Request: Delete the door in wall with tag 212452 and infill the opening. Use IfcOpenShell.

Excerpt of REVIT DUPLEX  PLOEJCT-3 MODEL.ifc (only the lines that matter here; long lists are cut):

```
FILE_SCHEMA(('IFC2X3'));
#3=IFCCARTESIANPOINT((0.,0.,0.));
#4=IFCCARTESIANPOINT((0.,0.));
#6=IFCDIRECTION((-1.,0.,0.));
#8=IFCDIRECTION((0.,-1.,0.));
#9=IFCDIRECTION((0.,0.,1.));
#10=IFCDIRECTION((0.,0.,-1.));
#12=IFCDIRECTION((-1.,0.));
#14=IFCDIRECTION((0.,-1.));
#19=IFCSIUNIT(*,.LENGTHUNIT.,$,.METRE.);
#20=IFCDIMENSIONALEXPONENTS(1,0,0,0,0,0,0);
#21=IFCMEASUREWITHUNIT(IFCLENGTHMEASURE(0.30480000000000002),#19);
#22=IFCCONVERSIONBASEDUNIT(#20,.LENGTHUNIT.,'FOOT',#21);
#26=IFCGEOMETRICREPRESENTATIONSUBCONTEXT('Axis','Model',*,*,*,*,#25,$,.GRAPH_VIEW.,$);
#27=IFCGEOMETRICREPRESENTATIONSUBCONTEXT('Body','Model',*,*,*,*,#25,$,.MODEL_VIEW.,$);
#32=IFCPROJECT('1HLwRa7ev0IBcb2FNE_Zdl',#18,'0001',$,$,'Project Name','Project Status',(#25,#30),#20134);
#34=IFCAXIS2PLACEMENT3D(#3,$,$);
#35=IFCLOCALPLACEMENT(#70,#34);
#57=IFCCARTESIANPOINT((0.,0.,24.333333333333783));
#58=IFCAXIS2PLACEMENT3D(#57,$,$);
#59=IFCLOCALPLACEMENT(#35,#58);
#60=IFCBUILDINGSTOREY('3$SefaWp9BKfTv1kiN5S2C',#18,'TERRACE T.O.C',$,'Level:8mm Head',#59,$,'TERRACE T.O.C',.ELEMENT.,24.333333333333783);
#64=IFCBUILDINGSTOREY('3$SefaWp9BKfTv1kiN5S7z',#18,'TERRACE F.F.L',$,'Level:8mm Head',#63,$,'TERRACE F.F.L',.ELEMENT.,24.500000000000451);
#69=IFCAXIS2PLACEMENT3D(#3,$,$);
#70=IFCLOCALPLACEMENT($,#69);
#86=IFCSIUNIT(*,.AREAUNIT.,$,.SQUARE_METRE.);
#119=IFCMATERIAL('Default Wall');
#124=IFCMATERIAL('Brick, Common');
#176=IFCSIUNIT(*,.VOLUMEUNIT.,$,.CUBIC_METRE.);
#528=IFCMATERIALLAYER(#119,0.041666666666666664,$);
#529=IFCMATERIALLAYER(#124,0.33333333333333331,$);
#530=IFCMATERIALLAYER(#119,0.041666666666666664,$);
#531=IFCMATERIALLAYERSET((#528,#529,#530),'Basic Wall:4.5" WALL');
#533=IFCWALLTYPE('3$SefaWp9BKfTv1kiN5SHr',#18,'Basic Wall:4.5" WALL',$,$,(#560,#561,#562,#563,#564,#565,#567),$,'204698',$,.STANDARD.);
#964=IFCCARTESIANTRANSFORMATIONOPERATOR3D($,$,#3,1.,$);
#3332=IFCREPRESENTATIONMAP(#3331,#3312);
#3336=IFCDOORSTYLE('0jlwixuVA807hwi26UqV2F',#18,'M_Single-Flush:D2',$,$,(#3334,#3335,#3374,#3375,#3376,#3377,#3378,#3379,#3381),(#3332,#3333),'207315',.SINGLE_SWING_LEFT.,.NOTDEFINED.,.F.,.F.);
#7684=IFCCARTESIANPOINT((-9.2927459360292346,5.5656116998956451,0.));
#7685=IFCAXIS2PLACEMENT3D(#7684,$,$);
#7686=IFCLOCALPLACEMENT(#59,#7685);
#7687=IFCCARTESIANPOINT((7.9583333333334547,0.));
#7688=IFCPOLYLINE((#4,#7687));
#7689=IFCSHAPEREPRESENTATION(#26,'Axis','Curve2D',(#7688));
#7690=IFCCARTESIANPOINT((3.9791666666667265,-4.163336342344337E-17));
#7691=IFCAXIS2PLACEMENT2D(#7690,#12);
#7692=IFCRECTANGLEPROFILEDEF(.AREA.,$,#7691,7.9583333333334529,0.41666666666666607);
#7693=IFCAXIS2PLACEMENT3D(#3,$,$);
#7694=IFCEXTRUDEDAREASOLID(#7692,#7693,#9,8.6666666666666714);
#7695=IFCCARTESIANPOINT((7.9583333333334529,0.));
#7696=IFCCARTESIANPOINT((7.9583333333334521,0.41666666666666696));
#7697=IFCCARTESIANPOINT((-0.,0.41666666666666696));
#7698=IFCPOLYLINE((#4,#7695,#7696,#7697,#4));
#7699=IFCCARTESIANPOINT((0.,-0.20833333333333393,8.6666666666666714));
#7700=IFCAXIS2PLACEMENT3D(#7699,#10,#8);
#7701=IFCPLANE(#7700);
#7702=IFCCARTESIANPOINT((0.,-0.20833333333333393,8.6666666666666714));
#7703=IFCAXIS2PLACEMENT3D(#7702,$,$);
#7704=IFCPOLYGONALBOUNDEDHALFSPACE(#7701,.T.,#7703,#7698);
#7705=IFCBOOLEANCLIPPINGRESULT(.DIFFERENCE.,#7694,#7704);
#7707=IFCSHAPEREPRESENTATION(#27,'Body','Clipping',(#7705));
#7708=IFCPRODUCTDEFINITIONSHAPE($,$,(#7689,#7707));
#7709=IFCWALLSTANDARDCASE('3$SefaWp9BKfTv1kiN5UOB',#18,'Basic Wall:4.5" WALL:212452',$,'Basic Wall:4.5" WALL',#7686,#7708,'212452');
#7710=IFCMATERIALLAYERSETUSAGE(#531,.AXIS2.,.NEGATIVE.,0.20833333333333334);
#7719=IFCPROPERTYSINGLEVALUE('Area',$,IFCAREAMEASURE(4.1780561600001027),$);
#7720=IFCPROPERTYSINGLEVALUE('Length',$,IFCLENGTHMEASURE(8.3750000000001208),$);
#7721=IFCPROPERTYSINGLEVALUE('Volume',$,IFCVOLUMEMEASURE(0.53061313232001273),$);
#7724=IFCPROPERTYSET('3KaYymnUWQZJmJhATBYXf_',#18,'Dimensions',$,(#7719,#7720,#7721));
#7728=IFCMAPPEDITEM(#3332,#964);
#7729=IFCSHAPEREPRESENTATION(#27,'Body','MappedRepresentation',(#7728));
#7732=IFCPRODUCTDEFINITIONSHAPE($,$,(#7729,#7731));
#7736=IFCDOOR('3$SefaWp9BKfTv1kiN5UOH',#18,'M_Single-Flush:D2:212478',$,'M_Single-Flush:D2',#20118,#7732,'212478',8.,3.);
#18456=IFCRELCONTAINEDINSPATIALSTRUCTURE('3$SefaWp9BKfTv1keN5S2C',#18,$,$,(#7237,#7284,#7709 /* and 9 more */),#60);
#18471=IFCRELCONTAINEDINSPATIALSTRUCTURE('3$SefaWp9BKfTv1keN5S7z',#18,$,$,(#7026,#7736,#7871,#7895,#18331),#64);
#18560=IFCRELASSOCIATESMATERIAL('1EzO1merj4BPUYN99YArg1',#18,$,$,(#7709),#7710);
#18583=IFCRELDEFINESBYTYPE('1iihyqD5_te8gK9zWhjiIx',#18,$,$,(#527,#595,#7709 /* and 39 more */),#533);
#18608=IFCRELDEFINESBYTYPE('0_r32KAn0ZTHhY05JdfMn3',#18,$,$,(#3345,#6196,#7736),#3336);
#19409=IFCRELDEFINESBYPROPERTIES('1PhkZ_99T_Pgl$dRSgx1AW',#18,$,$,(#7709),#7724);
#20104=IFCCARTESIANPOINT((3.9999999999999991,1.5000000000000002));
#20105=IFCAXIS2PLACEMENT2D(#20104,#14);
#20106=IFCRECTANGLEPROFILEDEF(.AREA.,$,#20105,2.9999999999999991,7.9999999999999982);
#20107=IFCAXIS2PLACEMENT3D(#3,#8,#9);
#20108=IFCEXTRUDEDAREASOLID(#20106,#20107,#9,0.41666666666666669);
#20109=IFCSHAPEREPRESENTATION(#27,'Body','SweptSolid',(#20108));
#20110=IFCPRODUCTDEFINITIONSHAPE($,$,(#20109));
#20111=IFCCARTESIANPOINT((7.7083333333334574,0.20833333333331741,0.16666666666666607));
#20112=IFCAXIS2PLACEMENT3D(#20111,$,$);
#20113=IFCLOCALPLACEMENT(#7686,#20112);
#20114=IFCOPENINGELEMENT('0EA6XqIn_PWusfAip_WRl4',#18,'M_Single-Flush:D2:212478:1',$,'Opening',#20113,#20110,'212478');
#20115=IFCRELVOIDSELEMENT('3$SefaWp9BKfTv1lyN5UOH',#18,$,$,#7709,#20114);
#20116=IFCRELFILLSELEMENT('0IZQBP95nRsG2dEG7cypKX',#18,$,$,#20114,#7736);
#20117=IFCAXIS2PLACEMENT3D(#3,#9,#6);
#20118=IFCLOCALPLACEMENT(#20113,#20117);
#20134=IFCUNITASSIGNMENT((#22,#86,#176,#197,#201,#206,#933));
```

```python
import ifcopenshell
import ifcopenshell.api.feature
import ifcopenshell.api.pset
import ifcopenshell.api.root
import ifcopenshell.geom
import ifcopenshell.util.element
import ifcopenshell.util.shape
import ifcopenshell.util.unit

model = ifcopenshell.open("REVIT DUPLEX  PLOEJCT-3 MODEL.ifc")
area_scale = ifcopenshell.util.unit.calculate_unit_scale(model, "AREAUNIT")
volume_scale = ifcopenshell.util.unit.calculate_unit_scale(model, "VOLUMEUNIT")
settings = ifcopenshell.geom.settings()


def volume(element):
    """Net volume in cubic metres, openings subtracted."""
    shape = ifcopenshell.geom.create_shape(settings, element)
    return ifcopenshell.util.shape.get_volume(shape.geometry)


door = model.by_guid("3$SefaWp9BKfTv1kiN5UOH")
opening = door.FillsVoids[0].RelatingOpeningElement
wall = opening.VoidsElements[0].RelatingBuildingElement
before = volume(wall)

ifcopenshell.api.root.remove_product(model, product=door)
ifcopenshell.api.feature.remove_feature(model, feature=opening)

after = volume(wall)
thickness = 0.127  # wall thickness in metres

# Update the wall's stored quantities.
pset = model.by_id(ifcopenshell.util.element.get_pset(wall, "Dimensions", should_inherit=False)["id"])
ifcopenshell.api.pset.edit_pset(model, pset=pset, properties={
    "Area": model.create_entity("IfcAreaMeasure", after / thickness / area_scale),
    "Volume": model.create_entity("IfcVolumeMeasure", after / volume_scale),
})

print(f"wall volume {before:.3f} -> {after:.3f} m3")

model.write("REVIT DUPLEX  PLOEJCT-3 MODEL_v2.ifc")
```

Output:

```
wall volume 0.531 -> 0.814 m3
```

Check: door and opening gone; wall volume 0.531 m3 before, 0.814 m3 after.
